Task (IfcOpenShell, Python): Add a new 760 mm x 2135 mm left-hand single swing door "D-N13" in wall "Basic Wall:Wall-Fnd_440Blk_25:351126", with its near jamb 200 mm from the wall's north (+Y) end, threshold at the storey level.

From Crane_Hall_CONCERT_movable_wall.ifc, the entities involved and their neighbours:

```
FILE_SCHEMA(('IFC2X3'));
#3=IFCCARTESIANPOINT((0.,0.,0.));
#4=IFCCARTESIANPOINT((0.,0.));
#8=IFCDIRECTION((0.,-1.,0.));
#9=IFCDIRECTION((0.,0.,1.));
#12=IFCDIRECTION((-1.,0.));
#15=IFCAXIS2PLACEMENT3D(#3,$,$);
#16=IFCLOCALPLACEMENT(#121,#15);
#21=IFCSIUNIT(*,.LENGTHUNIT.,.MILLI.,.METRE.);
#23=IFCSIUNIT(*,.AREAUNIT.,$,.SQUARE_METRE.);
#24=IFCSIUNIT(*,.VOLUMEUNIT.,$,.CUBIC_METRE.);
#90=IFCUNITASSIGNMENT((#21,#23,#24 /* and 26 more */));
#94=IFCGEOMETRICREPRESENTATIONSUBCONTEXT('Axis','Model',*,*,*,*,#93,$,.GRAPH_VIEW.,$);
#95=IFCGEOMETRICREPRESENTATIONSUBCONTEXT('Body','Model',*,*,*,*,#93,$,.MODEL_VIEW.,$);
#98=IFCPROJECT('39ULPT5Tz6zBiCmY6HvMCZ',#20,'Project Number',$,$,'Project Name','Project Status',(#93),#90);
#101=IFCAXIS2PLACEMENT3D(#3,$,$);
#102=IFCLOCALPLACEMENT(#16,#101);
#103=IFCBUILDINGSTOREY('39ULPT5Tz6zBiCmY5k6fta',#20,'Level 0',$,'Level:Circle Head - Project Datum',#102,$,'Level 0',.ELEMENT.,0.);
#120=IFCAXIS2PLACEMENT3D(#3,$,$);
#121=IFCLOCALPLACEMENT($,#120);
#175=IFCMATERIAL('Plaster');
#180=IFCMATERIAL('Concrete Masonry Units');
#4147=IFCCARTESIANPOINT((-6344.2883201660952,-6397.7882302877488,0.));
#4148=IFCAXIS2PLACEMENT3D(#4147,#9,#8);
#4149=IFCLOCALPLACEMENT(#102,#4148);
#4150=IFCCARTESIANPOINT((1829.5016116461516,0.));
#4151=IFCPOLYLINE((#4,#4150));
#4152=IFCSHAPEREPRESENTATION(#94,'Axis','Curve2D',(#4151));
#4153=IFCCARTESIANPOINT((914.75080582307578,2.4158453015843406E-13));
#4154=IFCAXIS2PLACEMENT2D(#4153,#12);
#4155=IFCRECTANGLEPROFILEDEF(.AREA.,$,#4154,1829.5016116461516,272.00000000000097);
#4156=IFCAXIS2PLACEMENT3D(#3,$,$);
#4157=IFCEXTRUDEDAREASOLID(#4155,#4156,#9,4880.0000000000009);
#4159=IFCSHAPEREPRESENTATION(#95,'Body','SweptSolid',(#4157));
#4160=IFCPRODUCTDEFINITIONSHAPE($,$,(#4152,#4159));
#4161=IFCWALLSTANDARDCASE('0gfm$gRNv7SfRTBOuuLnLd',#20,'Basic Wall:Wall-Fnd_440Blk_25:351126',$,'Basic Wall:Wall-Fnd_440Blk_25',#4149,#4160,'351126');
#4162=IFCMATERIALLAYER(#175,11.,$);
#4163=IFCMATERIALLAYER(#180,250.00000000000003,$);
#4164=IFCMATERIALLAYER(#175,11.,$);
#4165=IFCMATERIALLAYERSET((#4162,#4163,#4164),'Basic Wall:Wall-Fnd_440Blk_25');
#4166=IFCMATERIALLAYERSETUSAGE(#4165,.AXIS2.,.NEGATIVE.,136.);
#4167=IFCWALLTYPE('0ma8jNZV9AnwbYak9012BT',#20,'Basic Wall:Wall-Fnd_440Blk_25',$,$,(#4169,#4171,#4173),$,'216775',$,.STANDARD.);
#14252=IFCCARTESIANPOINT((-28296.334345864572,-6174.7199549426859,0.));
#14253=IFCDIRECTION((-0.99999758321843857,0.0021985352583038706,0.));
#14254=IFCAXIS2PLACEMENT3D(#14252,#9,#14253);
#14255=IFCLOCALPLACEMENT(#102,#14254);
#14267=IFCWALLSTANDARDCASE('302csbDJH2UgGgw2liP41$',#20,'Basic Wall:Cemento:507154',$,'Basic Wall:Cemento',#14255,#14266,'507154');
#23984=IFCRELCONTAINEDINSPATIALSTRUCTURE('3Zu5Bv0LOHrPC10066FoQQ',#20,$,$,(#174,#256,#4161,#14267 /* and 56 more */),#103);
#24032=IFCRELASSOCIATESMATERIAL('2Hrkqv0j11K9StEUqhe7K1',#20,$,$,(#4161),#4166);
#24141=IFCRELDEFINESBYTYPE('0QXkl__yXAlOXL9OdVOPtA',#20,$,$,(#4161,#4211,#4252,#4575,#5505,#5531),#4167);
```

```python
import numpy as np
import ifcopenshell
import ifcopenshell.api.feature
import ifcopenshell.api.geometry
import ifcopenshell.api.root
import ifcopenshell.api.spatial
import ifcopenshell.api.type
import ifcopenshell.geom
import ifcopenshell.util.element
import ifcopenshell.util.placement
import ifcopenshell.util.representation
import ifcopenshell.util.shape
import ifcopenshell.util.unit

model = ifcopenshell.open("Crane_Hall_CONCERT_movable_wall.ifc")
unit_scale = ifcopenshell.util.unit.calculate_unit_scale(model)
settings = ifcopenshell.geom.settings()


def volume(element):
    """Net volume in cubic metres, openings subtracted."""
    shape = ifcopenshell.geom.create_shape(settings, element)
    return ifcopenshell.util.shape.get_volume(shape.geometry)


wall = model.by_id(4161)
storey = ifcopenshell.util.element.get_container(wall, ifc_class="IfcBuildingStorey")
context = ifcopenshell.util.representation.get_context(model, "Model", "Body", "MODEL_VIEW")
before = volume(wall)

width, height, from_end, sill = 0.76, 2.135, 0.2, 0.0  # metres

# The wall runs along its own X axis, and the end named is its -X end.
wall_shape = ifcopenshell.geom.create_shape(settings, wall)
x, y, z = ifcopenshell.util.shape.get_vertices(wall_shape.geometry).T
start = x.min() + from_end
face, thickness = float(y.min()), float(y.max() - y.min())
wall_matrix = ifcopenshell.util.placement.get_local_placement(wall.ObjectPlacement)
level = ifcopenshell.util.placement.get_local_placement(storey.ObjectPlacement)[2, 3]


def in_wall(x, y):
    """Placement at x, y metres in the wall's axes, at sill height."""
    matrix = wall_matrix.copy()
    matrix[:, 3] = wall_matrix @ np.array([x / unit_scale, y / unit_scale, 0.0, 1.0])
    matrix[2, 3] = level + sill / unit_scale
    return matrix


# Opening: a box that overshoots both wall faces by 50 mm.
opening = ifcopenshell.api.root.create_entity(model, ifc_class="IfcOpeningElement")
box = ifcopenshell.api.geometry.add_wall_representation(
    model, context=context, length=width, height=height, thickness=thickness + 0.1
)
ifcopenshell.api.geometry.assign_representation(model, product=opening, representation=box)
ifcopenshell.api.geometry.edit_object_placement(model, product=opening, matrix=in_wall(start, face - 0.05), is_si=False)
ifcopenshell.api.feature.add_feature(model, feature=opening, element=wall)

door = ifcopenshell.api.root.create_entity(model, ifc_class="IfcDoor", name="D-N13")
door.OverallWidth, door.OverallHeight = width / unit_scale, height / unit_scale
body = ifcopenshell.api.geometry.add_door_representation(
    model,
    context=context,
    overall_width=door.OverallWidth,
    overall_height=door.OverallHeight,
    operation_type="SINGLE_SWING_LEFT",
    lining_properties={"LiningDepth": thickness / unit_scale, "ThresholdDepth": thickness / unit_scale},
)
ifcopenshell.api.geometry.assign_representation(model, product=door, representation=body)
ifcopenshell.api.spatial.assign_container(model, products=[door], relating_structure=storey)
fills = ifcopenshell.api.feature.add_filling(model, opening=opening, element=door)
fills.OwnerHistory = door.OwnerHistory  # required in IFC2X3

# IFC2X3 keeps the operation on the door style.
style = ifcopenshell.api.root.create_entity(model, ifc_class="IfcDoorStyle", name="D-N13")
style.OperationType, style.ConstructionType = "SINGLE_SWING_LEFT", "NOTDEFINED"
style.ParameterTakesPrecedence = style.Sizeable = False
ifcopenshell.api.type.assign_type(model, related_objects=[door], relating_type=style)

# The lining spans the wall, so the door starts at the wall face.
ifcopenshell.api.geometry.edit_object_placement(model, product=door, matrix=in_wall(start, face), is_si=False)

after = volume(wall)

print(f"wall volume {before:.3f} -> {after:.3f} m3")

model.write("Crane_Hall_CONCERT_movable_wall_v2.ifc")
```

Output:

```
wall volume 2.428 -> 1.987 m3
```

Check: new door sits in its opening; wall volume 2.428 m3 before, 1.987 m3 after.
